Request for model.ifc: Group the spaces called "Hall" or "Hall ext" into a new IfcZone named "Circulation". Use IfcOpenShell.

First a look at what the model holds.

```python
import ifcopenshell

model = ifcopenshell.open("model.ifc")
print(model.schema)
seen = {}
for space in model.by_type("IfcSpace"):
    seen[space.LongName] = seen.get(space.LongName, 0) + 1
for name, count in sorted(seen.items(), key=str):
    print(count, "x", name)
print("zones:", [z.Name for z in model.by_type("IfcZone")][:20])
```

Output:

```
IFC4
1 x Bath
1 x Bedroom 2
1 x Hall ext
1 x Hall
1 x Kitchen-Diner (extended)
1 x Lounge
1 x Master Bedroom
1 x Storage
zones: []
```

```python
import ifcopenshell
import ifcopenshell.api.group
import ifcopenshell.api.root

model = ifcopenshell.open("model.ifc")

names = {"Hall", "Hall ext"}
spaces = [s for s in model.by_type("IfcSpace") if s.LongName in names]

zone = ifcopenshell.api.root.create_entity(model, ifc_class="IfcZone", name="Circulation")
ifcopenshell.api.group.assign_group(model, products=spaces, group=zone)
print(len(spaces), "spaces in", zone.Name)

model.write("model_edited.ifc")
```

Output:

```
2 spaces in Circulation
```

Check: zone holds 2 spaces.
